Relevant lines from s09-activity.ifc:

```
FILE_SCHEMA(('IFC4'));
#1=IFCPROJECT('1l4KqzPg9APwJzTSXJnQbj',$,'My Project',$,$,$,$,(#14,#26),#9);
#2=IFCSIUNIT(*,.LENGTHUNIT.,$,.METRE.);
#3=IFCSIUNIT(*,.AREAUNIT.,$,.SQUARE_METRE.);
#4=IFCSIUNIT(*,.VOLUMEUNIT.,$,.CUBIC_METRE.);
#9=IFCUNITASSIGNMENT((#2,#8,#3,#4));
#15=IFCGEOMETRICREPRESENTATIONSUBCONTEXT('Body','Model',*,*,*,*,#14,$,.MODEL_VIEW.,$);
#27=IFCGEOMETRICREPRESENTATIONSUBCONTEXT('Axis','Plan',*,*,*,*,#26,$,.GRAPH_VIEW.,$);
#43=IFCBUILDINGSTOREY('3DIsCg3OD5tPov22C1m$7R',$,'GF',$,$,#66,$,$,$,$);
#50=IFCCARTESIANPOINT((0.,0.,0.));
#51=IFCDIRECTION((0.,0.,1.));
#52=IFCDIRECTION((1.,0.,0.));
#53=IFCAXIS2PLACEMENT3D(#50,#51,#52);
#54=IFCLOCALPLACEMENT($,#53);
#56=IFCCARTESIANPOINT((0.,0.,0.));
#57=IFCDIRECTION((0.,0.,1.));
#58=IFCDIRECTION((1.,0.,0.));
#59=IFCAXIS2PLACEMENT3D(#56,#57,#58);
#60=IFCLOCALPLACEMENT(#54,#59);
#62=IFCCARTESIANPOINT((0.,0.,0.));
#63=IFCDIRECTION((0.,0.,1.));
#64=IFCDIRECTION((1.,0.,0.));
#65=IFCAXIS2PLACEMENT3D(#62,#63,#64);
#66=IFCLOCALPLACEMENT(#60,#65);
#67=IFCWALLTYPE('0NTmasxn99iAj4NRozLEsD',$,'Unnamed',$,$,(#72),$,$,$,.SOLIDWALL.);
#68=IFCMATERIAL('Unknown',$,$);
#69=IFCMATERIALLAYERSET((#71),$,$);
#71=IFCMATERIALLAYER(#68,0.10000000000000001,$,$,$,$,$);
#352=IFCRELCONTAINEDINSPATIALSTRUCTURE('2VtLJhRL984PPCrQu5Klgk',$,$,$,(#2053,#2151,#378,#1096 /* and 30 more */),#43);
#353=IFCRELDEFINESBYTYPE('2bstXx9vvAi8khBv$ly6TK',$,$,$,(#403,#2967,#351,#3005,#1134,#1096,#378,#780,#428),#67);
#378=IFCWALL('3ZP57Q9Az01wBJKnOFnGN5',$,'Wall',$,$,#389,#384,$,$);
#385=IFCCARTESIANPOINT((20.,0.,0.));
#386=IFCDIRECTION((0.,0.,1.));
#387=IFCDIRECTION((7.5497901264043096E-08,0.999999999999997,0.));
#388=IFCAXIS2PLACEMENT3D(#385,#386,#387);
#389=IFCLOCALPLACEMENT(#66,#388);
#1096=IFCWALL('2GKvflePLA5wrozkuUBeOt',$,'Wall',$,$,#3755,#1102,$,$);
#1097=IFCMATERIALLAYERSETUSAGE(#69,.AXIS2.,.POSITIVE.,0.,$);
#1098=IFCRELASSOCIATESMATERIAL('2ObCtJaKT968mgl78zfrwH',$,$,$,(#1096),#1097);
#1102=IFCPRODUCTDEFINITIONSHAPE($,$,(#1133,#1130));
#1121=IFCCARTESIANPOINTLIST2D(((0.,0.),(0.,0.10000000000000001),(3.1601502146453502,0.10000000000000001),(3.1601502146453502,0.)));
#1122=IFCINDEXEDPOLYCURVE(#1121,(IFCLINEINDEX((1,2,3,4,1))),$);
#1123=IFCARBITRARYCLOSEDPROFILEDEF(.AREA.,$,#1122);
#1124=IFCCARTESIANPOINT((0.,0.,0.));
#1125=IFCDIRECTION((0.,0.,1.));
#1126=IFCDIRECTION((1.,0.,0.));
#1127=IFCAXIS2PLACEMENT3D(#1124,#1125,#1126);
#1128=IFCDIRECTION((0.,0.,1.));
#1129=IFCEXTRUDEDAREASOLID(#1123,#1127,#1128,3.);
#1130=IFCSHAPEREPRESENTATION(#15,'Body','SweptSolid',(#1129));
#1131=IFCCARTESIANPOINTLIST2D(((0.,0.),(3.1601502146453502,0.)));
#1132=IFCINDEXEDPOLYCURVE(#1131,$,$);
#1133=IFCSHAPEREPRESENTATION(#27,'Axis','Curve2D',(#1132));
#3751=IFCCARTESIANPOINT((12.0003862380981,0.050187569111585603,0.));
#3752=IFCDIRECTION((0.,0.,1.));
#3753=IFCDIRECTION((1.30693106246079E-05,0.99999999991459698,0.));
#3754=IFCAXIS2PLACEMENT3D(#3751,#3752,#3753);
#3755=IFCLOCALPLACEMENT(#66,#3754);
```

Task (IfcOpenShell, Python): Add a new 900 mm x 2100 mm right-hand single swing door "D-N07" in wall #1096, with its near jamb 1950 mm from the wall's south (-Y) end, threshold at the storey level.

```python
import numpy as np
import ifcopenshell
import ifcopenshell.api.feature
import ifcopenshell.api.geometry
import ifcopenshell.api.root
import ifcopenshell.api.spatial
import ifcopenshell.geom
import ifcopenshell.util.element
import ifcopenshell.util.placement
import ifcopenshell.util.representation
import ifcopenshell.util.shape
import ifcopenshell.util.unit

model = ifcopenshell.open("s09-activity.ifc")
unit_scale = ifcopenshell.util.unit.calculate_unit_scale(model)
settings = ifcopenshell.geom.settings()


def volume(element):
    """Net volume in cubic metres, openings subtracted."""
    shape = ifcopenshell.geom.create_shape(settings, element)
    return ifcopenshell.util.shape.get_volume(shape.geometry)


wall = model.by_guid("2GKvflePLA5wrozkuUBeOt")
storey = ifcopenshell.util.element.get_container(wall, ifc_class="IfcBuildingStorey")
context = ifcopenshell.util.representation.get_context(model, "Model", "Body", "MODEL_VIEW")
before = volume(wall)

width, height, from_end, sill = 0.9, 2.1, 1.95, 0.0  # metres

# The wall runs along its own X axis, and the end named is its -X end.
wall_shape = ifcopenshell.geom.create_shape(settings, wall)
x, y, z = ifcopenshell.util.shape.get_vertices(wall_shape.geometry).T
start = x.min() + from_end
face, thickness = float(y.min()), float(y.max() - y.min())
wall_matrix = ifcopenshell.util.placement.get_local_placement(wall.ObjectPlacement)
level = ifcopenshell.util.placement.get_local_placement(storey.ObjectPlacement)[2, 3]


def in_wall(x, y):
    """Placement at x, y metres in the wall's axes, at sill height."""
    matrix = wall_matrix.copy()
    matrix[:, 3] = wall_matrix @ np.array([x / unit_scale, y / unit_scale, 0.0, 1.0])
    matrix[2, 3] = level + sill / unit_scale
    return matrix


# Opening: a box that overshoots both wall faces by 50 mm.
opening = ifcopenshell.api.root.create_entity(model, ifc_class="IfcOpeningElement", predefined_type="OPENING")
box = ifcopenshell.api.geometry.add_wall_representation(
    model, context=context, length=width, height=height, thickness=thickness + 0.1
)
ifcopenshell.api.geometry.assign_representation(model, product=opening, representation=box)
ifcopenshell.api.geometry.edit_object_placement(model, product=opening, matrix=in_wall(start, face - 0.05), is_si=False)
ifcopenshell.api.feature.add_feature(model, feature=opening, element=wall)

door = ifcopenshell.api.root.create_entity(model, ifc_class="IfcDoor", name="D-N07", predefined_type="DOOR")
door.OverallWidth, door.OverallHeight = width / unit_scale, height / unit_scale
door.OperationType = "SINGLE_SWING_RIGHT"
body = ifcopenshell.api.geometry.add_door_representation(
    model,
    context=context,
    overall_width=door.OverallWidth,
    overall_height=door.OverallHeight,
    operation_type="SINGLE_SWING_RIGHT",
    lining_properties={"LiningDepth": thickness / unit_scale, "ThresholdDepth": thickness / unit_scale},
)
ifcopenshell.api.geometry.assign_representation(model, product=door, representation=body)
ifcopenshell.api.spatial.assign_container(model, products=[door], relating_structure=storey)
ifcopenshell.api.feature.add_filling(model, opening=opening, element=door)

# The lining spans the wall, so the door starts at the wall face.
ifcopenshell.api.geometry.edit_object_placement(model, product=door, matrix=in_wall(start, face), is_si=False)

after = volume(wall)

print(f"wall volume {before:.3f} -> {after:.3f} m3")

model.write("s09-activity-out.ifc")
```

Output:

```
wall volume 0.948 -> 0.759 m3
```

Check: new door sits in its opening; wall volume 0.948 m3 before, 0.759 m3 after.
